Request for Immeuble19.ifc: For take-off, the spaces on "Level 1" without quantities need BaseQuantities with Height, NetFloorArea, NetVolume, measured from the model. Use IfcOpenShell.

First a look at what the model holds.

```python
import ifcopenshell
import ifcopenshell.util.element
import ifcopenshell.util.unit

model = ifcopenshell.open("Immeuble19.ifc")
print(model.schema)
for unit_type in ("LENGTHUNIT", "AREAUNIT", "VOLUMEUNIT"):
    print(unit_type, ifcopenshell.util.unit.calculate_unit_scale(model, unit_type))
storey = next(s for s in model.by_type("IfcBuildingStorey") if s.Name == "Level 1")
spaces = [e for e in ifcopenshell.util.element.get_decomposition(storey) if e.is_a("IfcSpace")]
for e in sorted(spaces, key=lambda e: e.id()):
    print(e.id(), e.is_a(), e.Name, list(ifcopenshell.util.element.get_psets(e, qtos_only=True)), sep=" | ")
```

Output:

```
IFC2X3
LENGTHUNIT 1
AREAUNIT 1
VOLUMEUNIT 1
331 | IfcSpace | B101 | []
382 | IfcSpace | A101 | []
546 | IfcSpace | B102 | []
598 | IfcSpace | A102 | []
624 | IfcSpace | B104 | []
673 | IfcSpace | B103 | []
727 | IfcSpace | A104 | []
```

```python
import ifcopenshell
import ifcopenshell.api.pset
import ifcopenshell.geom
import ifcopenshell.util.element
import ifcopenshell.util.shape
import ifcopenshell.util.unit

model = ifcopenshell.open("Immeuble19.ifc")
unit_scale = ifcopenshell.util.unit.calculate_unit_scale(model)
area_scale = ifcopenshell.util.unit.calculate_unit_scale(model, "AREAUNIT")
volume_scale = ifcopenshell.util.unit.calculate_unit_scale(model, "VOLUMEUNIT")
settings = ifcopenshell.geom.settings()

storey = next(s for s in model.by_type("IfcBuildingStorey") if s.Name == "Level 1")
spaces = [e for e in ifcopenshell.util.element.get_decomposition(storey) if e.is_a("IfcSpace")]

for e in sorted(spaces, key=lambda e: e.id()):
    if ifcopenshell.util.element.get_psets(e, qtos_only=True, should_inherit=False):
        continue
    # Geometry comes back in metres, in the element's own axes.
    shape = ifcopenshell.geom.create_shape(settings, e)
    values = {
        "Height": ifcopenshell.util.shape.get_z(shape.geometry) / unit_scale,
        "NetFloorArea": ifcopenshell.util.shape.get_footprint_area(shape.geometry) / area_scale,
        "NetVolume": ifcopenshell.util.shape.get_volume(shape.geometry) / volume_scale,
    }
    qto = ifcopenshell.api.pset.add_qto(model, product=e, name="BaseQuantities")
    ifcopenshell.api.pset.edit_qto(model, qto=qto, properties=values)
    print(e.id(), {k: round(v, 3) for k, v in values.items()})

model.write("Immeuble19_v2.ifc")
```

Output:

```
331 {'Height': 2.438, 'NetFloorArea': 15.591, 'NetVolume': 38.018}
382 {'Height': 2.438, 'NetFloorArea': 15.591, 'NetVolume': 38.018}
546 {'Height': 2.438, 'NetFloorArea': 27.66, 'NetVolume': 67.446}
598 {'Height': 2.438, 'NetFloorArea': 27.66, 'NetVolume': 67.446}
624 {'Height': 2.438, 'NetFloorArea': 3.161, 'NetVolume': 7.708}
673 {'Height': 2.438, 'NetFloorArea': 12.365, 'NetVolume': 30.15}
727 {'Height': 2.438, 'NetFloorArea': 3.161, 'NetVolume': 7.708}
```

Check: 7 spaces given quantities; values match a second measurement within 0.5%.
